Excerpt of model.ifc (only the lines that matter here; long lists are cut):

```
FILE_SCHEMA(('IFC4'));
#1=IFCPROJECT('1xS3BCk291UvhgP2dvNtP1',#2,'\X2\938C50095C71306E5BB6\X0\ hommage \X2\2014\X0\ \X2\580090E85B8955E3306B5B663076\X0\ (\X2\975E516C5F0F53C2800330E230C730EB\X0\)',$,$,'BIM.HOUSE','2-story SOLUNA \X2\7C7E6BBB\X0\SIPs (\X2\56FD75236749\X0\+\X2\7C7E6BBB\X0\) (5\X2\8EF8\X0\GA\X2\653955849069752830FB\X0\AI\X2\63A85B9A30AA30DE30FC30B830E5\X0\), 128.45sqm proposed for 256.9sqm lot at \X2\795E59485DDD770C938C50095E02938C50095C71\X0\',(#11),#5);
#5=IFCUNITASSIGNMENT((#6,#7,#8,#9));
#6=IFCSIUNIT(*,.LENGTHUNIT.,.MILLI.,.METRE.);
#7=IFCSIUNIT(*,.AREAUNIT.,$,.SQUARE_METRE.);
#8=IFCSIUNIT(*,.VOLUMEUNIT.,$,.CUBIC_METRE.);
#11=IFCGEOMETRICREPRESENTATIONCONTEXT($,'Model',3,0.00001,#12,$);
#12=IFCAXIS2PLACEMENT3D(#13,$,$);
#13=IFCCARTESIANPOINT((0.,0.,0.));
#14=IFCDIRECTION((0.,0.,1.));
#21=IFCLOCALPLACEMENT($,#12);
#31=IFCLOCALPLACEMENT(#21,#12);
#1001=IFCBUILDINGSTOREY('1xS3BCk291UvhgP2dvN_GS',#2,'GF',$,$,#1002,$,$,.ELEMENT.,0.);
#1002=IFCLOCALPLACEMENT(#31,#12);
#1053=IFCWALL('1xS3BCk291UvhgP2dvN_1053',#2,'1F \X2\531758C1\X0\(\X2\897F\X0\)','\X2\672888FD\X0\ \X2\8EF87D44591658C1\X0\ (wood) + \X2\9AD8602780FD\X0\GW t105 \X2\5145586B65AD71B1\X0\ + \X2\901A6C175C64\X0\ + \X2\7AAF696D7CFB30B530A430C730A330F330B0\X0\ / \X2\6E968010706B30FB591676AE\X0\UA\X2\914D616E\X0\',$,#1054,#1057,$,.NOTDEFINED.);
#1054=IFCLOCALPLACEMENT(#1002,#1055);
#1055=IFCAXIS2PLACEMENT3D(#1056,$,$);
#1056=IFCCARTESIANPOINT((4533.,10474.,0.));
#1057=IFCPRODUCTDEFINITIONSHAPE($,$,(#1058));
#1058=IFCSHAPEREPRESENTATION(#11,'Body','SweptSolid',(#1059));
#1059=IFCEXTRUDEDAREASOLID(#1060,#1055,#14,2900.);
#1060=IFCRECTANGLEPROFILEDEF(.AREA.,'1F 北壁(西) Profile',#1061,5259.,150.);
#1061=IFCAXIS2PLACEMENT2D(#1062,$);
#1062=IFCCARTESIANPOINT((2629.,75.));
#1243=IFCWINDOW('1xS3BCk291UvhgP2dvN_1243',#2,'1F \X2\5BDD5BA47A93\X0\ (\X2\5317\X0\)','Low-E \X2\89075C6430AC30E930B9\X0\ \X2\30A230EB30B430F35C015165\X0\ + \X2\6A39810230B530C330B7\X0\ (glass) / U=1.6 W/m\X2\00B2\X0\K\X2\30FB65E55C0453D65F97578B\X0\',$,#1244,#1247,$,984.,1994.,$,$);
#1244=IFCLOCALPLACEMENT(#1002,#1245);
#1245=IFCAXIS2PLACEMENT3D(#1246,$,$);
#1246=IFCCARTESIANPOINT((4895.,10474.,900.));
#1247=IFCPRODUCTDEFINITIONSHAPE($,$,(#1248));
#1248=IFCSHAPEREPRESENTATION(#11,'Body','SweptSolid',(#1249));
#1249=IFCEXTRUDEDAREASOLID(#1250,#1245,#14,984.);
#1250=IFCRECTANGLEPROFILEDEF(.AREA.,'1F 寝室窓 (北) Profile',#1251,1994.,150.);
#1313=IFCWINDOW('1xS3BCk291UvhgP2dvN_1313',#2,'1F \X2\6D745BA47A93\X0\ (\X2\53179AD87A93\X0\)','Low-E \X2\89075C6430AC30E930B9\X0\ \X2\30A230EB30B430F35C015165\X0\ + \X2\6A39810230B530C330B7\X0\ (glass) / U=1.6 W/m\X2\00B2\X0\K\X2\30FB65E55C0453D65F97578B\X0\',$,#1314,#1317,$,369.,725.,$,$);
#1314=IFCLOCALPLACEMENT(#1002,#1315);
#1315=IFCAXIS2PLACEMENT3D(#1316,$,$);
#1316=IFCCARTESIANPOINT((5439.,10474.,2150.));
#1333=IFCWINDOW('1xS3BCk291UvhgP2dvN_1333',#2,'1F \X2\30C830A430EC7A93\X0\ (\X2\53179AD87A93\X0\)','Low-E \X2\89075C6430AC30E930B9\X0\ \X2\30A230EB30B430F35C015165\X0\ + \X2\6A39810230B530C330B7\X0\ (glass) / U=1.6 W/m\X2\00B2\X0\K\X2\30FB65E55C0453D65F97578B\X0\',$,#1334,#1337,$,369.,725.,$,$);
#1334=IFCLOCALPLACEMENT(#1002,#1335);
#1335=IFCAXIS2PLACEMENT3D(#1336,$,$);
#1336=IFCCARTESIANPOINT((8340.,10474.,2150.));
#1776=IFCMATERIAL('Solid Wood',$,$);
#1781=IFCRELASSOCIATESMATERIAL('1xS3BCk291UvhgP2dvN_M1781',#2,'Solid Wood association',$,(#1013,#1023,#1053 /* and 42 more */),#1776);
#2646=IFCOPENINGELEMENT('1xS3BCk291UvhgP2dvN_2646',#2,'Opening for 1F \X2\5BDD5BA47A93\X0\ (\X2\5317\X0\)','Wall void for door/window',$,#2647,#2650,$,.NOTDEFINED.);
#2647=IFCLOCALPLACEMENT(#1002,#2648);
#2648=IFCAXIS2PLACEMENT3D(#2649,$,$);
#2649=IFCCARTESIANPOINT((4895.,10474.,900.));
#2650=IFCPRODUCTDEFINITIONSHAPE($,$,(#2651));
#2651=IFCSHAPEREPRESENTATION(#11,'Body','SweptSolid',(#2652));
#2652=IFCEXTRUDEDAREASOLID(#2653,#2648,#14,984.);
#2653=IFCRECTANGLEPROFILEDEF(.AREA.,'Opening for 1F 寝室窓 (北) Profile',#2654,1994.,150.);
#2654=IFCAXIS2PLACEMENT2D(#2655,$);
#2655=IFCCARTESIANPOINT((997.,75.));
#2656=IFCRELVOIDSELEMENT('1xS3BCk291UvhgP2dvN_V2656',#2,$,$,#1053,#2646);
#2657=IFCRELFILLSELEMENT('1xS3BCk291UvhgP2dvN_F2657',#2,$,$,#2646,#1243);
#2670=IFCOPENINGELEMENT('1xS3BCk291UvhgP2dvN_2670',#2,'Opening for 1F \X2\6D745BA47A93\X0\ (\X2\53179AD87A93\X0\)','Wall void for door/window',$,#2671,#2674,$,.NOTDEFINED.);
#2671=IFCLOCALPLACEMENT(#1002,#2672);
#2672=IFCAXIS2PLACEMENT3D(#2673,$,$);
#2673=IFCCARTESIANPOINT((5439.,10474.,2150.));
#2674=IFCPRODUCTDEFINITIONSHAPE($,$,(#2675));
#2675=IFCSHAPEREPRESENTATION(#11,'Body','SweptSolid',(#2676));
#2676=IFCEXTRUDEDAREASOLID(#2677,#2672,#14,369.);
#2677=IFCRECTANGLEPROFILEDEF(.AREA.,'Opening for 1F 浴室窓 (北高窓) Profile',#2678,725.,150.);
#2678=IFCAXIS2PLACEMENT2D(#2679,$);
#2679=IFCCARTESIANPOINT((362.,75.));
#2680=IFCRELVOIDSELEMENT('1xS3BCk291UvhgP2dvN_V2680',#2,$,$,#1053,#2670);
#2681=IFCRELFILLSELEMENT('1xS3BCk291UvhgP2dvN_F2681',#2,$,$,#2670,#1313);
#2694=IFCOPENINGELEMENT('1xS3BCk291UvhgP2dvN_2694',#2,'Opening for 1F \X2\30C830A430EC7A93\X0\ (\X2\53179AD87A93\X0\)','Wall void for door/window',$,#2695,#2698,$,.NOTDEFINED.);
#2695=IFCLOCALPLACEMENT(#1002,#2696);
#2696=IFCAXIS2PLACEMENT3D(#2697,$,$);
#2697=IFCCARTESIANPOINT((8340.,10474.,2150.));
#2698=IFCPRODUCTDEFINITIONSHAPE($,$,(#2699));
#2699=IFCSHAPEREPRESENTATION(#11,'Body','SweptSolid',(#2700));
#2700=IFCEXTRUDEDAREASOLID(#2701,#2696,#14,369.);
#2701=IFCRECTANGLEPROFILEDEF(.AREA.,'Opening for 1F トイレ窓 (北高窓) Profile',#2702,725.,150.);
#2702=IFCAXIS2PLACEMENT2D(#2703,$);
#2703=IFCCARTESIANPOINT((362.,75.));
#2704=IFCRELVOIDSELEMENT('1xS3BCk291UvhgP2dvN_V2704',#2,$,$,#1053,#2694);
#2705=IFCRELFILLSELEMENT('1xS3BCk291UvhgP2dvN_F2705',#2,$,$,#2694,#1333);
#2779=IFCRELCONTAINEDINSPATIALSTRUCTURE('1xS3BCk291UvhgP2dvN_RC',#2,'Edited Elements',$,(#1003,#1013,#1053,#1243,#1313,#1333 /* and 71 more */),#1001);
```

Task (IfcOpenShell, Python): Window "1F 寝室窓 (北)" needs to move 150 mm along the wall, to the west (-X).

```python
import ifcopenshell
import ifcopenshell.api.geometry
import ifcopenshell.util.placement

model = ifcopenshell.open("model.ifc")

window = model.by_guid("1xS3BCk291UvhgP2dvN_1243")
opening = window.FillsVoids[0].RelatingOpeningElement
wall = opening.VoidsElements[0].RelatingBuildingElement

wall_matrix = ifcopenshell.util.placement.get_local_placement(wall.ObjectPlacement)
shift = wall_matrix[:3, 0] * -150.0
before = ifcopenshell.util.placement.get_local_placement(window.ObjectPlacement)[:3, 3].copy()

# The window is not placed relative to its opening, so move both.
for product in (opening, window):
    matrix = ifcopenshell.util.placement.get_local_placement(product.ObjectPlacement)
    matrix[:3, 3] += shift
    ifcopenshell.api.geometry.edit_object_placement(model, product=product, matrix=matrix, is_si=False)

after = ifcopenshell.util.placement.get_local_placement(window.ObjectPlacement)[:3, 3]
print("window moved by", (after - before).round(3) + 0.0)

model.write("model_edited.ifc")
```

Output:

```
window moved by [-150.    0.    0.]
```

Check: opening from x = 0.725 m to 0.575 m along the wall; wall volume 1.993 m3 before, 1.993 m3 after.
